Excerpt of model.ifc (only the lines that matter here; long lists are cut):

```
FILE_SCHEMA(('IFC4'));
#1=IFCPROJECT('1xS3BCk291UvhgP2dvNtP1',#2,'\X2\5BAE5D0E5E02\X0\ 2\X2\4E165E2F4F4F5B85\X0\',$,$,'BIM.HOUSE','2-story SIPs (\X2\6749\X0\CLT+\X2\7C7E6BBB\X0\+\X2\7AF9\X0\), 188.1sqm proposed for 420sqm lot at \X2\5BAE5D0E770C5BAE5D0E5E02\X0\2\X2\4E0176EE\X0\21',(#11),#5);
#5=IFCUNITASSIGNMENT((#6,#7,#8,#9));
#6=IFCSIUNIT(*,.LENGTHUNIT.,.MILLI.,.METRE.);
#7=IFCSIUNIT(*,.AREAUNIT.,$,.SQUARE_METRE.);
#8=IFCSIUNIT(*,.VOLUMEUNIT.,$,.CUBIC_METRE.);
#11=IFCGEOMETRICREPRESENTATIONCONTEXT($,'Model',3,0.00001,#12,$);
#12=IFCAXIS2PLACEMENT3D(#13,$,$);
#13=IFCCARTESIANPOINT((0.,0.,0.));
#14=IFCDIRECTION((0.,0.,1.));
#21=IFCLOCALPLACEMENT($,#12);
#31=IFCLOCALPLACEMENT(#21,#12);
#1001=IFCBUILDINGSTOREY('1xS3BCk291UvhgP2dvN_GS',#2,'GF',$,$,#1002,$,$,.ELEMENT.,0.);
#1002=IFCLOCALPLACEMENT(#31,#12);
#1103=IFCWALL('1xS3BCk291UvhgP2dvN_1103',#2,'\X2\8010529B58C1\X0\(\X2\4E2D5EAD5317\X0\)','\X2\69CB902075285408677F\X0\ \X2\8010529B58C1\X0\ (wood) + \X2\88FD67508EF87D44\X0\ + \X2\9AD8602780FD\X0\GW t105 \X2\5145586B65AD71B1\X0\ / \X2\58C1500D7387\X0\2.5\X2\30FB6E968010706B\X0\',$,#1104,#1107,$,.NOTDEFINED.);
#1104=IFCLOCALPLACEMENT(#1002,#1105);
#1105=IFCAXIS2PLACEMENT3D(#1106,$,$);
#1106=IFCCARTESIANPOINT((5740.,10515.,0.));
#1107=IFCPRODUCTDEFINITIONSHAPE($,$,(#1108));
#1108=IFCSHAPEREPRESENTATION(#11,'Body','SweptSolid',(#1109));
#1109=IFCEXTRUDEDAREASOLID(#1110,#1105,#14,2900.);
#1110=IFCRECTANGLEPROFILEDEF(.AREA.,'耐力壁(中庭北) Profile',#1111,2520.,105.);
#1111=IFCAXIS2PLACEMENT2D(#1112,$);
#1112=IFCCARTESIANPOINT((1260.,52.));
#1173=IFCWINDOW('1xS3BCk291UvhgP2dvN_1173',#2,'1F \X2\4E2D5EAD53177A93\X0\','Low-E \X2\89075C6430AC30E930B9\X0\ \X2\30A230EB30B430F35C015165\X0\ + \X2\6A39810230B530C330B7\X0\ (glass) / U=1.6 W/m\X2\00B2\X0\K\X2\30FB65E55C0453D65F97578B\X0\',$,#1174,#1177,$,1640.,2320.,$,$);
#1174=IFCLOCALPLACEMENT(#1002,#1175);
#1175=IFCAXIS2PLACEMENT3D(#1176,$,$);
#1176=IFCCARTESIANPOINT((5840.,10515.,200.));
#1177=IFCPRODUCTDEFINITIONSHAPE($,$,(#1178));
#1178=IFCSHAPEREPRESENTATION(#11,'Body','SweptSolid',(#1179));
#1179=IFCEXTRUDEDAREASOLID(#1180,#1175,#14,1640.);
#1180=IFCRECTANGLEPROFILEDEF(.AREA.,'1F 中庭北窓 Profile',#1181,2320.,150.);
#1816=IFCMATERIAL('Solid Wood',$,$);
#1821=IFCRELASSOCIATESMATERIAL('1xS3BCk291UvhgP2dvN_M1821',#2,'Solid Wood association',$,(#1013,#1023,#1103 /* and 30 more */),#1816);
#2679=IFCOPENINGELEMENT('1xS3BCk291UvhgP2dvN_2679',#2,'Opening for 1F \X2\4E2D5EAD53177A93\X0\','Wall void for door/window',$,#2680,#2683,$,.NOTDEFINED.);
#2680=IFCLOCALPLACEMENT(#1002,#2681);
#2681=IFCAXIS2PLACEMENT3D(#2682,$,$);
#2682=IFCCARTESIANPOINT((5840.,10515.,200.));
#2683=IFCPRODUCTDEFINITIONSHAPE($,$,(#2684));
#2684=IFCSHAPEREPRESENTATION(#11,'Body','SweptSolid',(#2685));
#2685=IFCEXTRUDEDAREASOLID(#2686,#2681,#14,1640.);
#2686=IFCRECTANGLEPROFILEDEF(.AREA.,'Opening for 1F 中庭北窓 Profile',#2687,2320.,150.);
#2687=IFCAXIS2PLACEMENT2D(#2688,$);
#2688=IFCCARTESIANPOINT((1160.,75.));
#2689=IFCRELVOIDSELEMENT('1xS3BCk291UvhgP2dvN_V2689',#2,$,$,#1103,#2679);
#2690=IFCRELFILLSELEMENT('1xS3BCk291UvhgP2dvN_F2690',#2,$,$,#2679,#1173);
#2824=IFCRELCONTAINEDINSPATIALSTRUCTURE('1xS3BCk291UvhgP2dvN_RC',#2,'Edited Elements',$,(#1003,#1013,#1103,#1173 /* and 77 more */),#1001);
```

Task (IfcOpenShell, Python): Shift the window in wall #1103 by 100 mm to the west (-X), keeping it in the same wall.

```python
import ifcopenshell
import ifcopenshell.api.geometry
import ifcopenshell.util.placement

model = ifcopenshell.open("model.ifc")

window = model.by_id(1173)
opening = window.FillsVoids[0].RelatingOpeningElement
wall = opening.VoidsElements[0].RelatingBuildingElement

wall_matrix = ifcopenshell.util.placement.get_local_placement(wall.ObjectPlacement)
shift = wall_matrix[:3, 0] * -100.0
before = ifcopenshell.util.placement.get_local_placement(window.ObjectPlacement)[:3, 3].copy()

# The window is not placed relative to its opening, so move both.
for product in (opening, window):
    matrix = ifcopenshell.util.placement.get_local_placement(product.ObjectPlacement)
    matrix[:3, 3] += shift
    ifcopenshell.api.geometry.edit_object_placement(model, product=product, matrix=matrix, is_si=False)

after = ifcopenshell.util.placement.get_local_placement(window.ObjectPlacement)[:3, 3]
print("window moved by", (after - before).round(3) + 0.0)

model.write("model_edited.ifc")
```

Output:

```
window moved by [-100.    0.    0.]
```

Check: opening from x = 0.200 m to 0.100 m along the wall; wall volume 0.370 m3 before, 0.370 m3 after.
